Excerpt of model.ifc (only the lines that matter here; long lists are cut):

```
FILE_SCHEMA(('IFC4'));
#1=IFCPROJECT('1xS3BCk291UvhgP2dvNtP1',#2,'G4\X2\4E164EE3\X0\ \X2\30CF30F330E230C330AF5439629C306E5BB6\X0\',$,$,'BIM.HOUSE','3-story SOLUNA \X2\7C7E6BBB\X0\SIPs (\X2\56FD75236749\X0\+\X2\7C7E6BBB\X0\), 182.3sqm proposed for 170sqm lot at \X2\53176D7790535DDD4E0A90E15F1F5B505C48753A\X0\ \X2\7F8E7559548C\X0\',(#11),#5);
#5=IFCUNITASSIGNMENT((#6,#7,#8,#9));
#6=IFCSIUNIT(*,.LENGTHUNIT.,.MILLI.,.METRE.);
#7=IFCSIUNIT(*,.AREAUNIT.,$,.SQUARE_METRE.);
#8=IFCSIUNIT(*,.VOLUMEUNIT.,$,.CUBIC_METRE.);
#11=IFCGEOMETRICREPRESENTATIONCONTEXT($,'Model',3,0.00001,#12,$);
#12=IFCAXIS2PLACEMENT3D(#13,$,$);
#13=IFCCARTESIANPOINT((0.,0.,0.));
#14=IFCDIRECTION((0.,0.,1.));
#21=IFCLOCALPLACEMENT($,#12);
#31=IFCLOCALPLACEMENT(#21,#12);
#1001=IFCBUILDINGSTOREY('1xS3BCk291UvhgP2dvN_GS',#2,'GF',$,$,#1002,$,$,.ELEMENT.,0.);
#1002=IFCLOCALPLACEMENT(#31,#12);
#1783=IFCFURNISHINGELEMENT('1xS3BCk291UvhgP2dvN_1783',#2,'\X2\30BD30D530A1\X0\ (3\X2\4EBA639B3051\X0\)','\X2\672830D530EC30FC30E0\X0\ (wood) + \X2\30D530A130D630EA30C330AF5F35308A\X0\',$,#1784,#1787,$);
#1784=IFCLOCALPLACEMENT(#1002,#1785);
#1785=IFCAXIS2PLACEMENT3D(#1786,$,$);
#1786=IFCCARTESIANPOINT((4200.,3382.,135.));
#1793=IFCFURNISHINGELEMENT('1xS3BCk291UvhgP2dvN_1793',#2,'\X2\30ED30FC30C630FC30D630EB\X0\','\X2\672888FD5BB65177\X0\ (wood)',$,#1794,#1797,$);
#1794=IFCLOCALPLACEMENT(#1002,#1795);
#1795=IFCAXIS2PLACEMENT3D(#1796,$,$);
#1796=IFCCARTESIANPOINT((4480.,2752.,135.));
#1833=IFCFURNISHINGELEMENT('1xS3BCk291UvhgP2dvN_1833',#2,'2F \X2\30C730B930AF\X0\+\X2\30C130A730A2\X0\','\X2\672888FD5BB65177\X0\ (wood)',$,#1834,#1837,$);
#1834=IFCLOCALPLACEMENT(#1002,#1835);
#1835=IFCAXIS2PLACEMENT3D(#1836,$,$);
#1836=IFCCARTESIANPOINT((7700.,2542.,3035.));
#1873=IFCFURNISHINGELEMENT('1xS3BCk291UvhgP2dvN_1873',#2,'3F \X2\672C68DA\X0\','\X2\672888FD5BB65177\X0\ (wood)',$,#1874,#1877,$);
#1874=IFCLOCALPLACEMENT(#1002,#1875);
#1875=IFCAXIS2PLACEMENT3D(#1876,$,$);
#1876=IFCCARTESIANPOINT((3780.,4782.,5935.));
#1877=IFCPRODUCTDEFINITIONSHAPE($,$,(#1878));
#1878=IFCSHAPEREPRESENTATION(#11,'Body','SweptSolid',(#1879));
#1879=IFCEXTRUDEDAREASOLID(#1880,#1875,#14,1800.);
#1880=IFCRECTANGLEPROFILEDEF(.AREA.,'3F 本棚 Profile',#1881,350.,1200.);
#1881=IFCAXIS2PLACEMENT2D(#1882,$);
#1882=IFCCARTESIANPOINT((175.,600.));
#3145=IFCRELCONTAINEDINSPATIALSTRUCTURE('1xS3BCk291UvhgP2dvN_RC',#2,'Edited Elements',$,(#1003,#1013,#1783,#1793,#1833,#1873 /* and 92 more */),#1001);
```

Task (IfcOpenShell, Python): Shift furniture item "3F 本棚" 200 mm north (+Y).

```python
import ifcopenshell
import ifcopenshell.api.geometry
import ifcopenshell.util.placement
import ifcopenshell.util.unit

model = ifcopenshell.open("model.ifc")
unit_scale = ifcopenshell.util.unit.calculate_unit_scale(model)

item = model.by_id(1873)
matrix = ifcopenshell.util.placement.get_local_placement(item.ObjectPlacement)
matrix[1, 3] += 0.2 / unit_scale
ifcopenshell.api.geometry.edit_object_placement(model, product=item, matrix=matrix, is_si=False)

print(ifcopenshell.util.placement.get_local_placement(item.ObjectPlacement).round(3) + 0.0)

model.write("model-out.ifc")
```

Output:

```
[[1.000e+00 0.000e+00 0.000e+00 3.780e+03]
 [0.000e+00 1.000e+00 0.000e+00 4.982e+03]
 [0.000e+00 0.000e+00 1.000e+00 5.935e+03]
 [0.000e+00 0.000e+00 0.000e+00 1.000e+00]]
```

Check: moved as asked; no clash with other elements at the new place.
